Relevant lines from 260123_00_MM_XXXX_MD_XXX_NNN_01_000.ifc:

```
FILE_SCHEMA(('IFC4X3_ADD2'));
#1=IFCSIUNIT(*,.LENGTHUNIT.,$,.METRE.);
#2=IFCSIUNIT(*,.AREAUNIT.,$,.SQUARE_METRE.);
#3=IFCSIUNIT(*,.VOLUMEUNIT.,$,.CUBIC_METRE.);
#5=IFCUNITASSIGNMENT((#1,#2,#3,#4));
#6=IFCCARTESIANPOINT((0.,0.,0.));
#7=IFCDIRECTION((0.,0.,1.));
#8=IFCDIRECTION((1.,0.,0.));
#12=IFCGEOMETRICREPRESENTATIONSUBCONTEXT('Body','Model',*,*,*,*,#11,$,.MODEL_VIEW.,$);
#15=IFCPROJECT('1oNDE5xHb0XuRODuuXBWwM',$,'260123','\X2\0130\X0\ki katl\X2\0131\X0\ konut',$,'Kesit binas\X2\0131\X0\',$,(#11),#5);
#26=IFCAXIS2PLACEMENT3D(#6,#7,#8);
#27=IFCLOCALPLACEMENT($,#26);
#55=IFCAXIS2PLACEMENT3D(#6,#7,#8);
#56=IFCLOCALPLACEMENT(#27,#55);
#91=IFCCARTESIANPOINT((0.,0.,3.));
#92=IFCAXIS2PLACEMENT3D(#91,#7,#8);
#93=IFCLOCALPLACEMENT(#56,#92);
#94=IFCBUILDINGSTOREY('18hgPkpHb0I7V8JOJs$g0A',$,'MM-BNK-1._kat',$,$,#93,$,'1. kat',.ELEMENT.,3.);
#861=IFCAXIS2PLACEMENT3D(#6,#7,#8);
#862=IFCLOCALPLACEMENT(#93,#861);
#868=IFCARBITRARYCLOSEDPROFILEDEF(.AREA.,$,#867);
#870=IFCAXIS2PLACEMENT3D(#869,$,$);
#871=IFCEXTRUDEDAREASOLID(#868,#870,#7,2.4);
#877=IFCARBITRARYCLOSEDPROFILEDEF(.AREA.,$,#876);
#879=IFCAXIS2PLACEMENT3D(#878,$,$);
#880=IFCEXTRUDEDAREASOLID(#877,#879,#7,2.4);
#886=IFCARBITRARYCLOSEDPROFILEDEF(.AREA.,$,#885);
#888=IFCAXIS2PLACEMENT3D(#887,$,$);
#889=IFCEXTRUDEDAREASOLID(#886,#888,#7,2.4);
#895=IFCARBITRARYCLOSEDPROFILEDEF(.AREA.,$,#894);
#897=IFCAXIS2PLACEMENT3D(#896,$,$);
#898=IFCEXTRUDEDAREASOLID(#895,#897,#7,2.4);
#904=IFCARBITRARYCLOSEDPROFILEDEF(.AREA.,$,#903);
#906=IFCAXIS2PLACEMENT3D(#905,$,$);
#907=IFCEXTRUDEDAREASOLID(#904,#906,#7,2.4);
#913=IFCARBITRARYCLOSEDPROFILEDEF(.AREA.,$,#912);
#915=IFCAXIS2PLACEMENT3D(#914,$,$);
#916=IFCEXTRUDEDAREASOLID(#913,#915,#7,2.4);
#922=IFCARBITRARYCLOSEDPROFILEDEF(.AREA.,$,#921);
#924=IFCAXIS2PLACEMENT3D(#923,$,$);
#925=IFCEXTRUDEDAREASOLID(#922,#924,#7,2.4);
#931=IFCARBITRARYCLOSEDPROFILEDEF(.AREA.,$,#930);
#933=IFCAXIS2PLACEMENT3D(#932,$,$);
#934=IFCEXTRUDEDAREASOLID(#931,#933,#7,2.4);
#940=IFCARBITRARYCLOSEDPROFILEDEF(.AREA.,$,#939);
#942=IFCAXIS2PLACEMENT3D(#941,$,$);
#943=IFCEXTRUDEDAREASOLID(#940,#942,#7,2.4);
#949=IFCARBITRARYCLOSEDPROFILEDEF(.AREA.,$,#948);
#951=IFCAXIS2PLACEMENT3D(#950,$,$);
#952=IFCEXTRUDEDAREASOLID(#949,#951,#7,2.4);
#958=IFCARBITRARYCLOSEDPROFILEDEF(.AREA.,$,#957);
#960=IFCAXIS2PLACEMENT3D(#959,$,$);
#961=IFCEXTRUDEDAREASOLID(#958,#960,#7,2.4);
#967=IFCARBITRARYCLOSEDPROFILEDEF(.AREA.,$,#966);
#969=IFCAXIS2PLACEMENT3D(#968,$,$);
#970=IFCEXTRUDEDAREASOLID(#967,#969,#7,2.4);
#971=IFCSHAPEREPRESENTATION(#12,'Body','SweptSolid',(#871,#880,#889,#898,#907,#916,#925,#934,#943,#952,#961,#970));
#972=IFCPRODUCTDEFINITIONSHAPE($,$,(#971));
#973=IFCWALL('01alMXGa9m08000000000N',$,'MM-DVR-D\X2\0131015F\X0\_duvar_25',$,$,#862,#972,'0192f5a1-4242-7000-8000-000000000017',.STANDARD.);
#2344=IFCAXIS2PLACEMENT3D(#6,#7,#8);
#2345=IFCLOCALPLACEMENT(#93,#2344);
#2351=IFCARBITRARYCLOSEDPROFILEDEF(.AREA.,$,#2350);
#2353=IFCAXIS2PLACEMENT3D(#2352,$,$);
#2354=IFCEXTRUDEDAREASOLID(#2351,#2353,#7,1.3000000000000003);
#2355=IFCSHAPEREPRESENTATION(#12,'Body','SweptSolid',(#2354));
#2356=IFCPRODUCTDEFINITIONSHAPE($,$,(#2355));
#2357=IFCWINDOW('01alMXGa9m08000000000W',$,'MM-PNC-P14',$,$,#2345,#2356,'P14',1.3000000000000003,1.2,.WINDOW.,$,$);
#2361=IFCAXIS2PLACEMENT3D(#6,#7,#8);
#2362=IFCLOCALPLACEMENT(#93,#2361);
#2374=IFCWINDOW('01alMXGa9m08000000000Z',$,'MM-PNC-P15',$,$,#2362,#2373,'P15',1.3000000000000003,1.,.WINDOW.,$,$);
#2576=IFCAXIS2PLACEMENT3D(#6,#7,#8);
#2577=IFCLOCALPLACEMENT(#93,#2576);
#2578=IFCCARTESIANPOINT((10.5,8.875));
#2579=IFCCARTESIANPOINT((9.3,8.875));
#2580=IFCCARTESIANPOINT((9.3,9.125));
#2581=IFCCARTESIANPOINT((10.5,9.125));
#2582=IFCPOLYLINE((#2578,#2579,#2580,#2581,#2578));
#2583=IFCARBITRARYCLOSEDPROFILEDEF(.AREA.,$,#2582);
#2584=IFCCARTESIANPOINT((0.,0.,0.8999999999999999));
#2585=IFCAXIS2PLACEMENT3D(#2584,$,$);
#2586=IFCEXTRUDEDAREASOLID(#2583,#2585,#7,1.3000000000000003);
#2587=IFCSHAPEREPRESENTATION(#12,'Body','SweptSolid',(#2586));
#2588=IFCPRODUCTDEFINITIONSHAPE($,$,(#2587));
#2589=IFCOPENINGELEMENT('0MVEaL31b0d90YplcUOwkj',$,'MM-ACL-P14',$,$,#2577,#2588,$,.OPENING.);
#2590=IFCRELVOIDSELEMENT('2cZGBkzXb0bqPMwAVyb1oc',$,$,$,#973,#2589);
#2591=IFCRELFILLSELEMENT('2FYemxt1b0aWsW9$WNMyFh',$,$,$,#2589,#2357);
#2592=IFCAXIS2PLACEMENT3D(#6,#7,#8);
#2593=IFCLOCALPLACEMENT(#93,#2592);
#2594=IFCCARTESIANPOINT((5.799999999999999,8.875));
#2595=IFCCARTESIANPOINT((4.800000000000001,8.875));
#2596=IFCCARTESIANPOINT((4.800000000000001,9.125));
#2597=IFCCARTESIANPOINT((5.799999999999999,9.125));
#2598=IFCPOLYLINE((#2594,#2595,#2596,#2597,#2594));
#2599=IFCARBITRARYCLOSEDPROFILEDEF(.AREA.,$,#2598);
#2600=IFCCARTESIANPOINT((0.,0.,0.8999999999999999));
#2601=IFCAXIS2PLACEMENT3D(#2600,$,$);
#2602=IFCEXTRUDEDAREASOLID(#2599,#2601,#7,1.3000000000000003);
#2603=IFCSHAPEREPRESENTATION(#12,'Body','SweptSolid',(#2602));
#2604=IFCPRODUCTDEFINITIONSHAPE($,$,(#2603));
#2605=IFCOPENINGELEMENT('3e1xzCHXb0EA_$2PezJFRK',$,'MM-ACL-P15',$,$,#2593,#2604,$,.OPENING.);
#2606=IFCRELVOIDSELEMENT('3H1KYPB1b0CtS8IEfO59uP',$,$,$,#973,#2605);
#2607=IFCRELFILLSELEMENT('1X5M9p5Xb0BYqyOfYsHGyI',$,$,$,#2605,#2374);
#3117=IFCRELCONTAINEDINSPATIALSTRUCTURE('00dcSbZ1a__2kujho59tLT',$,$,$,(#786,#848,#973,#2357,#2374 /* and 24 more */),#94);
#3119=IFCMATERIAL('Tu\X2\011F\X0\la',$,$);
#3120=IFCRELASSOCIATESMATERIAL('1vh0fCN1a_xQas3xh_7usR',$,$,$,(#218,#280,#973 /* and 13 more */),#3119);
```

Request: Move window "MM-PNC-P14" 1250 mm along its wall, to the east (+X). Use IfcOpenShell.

```python
import ifcopenshell
import ifcopenshell.api.geometry
import ifcopenshell.util.placement
import ifcopenshell.util.unit

model = ifcopenshell.open("260123_00_MM_XXXX_MD_XXX_NNN_01_000.ifc")
unit_scale = ifcopenshell.util.unit.calculate_unit_scale(model)

window = model.by_guid("01alMXGa9m08000000000W")
opening = window.FillsVoids[0].RelatingOpeningElement
wall = opening.VoidsElements[0].RelatingBuildingElement

wall_matrix = ifcopenshell.util.placement.get_local_placement(wall.ObjectPlacement)
shift = wall_matrix[:3, 0] * 1.25 / unit_scale
before = ifcopenshell.util.placement.get_local_placement(window.ObjectPlacement)[:3, 3].copy()

# The window is not placed relative to its opening, so move both.
for product in (opening, window):
    matrix = ifcopenshell.util.placement.get_local_placement(product.ObjectPlacement)
    matrix[:3, 3] += shift
    ifcopenshell.api.geometry.edit_object_placement(model, product=product, matrix=matrix, is_si=False)

after = ifcopenshell.util.placement.get_local_placement(window.ObjectPlacement)[:3, 3]
print("window moved by", (after - before).round(3) + 0.0)

model.write("260123_00_MM_XXXX_MD_XXX_NNN_01_000_edited.ifc")
```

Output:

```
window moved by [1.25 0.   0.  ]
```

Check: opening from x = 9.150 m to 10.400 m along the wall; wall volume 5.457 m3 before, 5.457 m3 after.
